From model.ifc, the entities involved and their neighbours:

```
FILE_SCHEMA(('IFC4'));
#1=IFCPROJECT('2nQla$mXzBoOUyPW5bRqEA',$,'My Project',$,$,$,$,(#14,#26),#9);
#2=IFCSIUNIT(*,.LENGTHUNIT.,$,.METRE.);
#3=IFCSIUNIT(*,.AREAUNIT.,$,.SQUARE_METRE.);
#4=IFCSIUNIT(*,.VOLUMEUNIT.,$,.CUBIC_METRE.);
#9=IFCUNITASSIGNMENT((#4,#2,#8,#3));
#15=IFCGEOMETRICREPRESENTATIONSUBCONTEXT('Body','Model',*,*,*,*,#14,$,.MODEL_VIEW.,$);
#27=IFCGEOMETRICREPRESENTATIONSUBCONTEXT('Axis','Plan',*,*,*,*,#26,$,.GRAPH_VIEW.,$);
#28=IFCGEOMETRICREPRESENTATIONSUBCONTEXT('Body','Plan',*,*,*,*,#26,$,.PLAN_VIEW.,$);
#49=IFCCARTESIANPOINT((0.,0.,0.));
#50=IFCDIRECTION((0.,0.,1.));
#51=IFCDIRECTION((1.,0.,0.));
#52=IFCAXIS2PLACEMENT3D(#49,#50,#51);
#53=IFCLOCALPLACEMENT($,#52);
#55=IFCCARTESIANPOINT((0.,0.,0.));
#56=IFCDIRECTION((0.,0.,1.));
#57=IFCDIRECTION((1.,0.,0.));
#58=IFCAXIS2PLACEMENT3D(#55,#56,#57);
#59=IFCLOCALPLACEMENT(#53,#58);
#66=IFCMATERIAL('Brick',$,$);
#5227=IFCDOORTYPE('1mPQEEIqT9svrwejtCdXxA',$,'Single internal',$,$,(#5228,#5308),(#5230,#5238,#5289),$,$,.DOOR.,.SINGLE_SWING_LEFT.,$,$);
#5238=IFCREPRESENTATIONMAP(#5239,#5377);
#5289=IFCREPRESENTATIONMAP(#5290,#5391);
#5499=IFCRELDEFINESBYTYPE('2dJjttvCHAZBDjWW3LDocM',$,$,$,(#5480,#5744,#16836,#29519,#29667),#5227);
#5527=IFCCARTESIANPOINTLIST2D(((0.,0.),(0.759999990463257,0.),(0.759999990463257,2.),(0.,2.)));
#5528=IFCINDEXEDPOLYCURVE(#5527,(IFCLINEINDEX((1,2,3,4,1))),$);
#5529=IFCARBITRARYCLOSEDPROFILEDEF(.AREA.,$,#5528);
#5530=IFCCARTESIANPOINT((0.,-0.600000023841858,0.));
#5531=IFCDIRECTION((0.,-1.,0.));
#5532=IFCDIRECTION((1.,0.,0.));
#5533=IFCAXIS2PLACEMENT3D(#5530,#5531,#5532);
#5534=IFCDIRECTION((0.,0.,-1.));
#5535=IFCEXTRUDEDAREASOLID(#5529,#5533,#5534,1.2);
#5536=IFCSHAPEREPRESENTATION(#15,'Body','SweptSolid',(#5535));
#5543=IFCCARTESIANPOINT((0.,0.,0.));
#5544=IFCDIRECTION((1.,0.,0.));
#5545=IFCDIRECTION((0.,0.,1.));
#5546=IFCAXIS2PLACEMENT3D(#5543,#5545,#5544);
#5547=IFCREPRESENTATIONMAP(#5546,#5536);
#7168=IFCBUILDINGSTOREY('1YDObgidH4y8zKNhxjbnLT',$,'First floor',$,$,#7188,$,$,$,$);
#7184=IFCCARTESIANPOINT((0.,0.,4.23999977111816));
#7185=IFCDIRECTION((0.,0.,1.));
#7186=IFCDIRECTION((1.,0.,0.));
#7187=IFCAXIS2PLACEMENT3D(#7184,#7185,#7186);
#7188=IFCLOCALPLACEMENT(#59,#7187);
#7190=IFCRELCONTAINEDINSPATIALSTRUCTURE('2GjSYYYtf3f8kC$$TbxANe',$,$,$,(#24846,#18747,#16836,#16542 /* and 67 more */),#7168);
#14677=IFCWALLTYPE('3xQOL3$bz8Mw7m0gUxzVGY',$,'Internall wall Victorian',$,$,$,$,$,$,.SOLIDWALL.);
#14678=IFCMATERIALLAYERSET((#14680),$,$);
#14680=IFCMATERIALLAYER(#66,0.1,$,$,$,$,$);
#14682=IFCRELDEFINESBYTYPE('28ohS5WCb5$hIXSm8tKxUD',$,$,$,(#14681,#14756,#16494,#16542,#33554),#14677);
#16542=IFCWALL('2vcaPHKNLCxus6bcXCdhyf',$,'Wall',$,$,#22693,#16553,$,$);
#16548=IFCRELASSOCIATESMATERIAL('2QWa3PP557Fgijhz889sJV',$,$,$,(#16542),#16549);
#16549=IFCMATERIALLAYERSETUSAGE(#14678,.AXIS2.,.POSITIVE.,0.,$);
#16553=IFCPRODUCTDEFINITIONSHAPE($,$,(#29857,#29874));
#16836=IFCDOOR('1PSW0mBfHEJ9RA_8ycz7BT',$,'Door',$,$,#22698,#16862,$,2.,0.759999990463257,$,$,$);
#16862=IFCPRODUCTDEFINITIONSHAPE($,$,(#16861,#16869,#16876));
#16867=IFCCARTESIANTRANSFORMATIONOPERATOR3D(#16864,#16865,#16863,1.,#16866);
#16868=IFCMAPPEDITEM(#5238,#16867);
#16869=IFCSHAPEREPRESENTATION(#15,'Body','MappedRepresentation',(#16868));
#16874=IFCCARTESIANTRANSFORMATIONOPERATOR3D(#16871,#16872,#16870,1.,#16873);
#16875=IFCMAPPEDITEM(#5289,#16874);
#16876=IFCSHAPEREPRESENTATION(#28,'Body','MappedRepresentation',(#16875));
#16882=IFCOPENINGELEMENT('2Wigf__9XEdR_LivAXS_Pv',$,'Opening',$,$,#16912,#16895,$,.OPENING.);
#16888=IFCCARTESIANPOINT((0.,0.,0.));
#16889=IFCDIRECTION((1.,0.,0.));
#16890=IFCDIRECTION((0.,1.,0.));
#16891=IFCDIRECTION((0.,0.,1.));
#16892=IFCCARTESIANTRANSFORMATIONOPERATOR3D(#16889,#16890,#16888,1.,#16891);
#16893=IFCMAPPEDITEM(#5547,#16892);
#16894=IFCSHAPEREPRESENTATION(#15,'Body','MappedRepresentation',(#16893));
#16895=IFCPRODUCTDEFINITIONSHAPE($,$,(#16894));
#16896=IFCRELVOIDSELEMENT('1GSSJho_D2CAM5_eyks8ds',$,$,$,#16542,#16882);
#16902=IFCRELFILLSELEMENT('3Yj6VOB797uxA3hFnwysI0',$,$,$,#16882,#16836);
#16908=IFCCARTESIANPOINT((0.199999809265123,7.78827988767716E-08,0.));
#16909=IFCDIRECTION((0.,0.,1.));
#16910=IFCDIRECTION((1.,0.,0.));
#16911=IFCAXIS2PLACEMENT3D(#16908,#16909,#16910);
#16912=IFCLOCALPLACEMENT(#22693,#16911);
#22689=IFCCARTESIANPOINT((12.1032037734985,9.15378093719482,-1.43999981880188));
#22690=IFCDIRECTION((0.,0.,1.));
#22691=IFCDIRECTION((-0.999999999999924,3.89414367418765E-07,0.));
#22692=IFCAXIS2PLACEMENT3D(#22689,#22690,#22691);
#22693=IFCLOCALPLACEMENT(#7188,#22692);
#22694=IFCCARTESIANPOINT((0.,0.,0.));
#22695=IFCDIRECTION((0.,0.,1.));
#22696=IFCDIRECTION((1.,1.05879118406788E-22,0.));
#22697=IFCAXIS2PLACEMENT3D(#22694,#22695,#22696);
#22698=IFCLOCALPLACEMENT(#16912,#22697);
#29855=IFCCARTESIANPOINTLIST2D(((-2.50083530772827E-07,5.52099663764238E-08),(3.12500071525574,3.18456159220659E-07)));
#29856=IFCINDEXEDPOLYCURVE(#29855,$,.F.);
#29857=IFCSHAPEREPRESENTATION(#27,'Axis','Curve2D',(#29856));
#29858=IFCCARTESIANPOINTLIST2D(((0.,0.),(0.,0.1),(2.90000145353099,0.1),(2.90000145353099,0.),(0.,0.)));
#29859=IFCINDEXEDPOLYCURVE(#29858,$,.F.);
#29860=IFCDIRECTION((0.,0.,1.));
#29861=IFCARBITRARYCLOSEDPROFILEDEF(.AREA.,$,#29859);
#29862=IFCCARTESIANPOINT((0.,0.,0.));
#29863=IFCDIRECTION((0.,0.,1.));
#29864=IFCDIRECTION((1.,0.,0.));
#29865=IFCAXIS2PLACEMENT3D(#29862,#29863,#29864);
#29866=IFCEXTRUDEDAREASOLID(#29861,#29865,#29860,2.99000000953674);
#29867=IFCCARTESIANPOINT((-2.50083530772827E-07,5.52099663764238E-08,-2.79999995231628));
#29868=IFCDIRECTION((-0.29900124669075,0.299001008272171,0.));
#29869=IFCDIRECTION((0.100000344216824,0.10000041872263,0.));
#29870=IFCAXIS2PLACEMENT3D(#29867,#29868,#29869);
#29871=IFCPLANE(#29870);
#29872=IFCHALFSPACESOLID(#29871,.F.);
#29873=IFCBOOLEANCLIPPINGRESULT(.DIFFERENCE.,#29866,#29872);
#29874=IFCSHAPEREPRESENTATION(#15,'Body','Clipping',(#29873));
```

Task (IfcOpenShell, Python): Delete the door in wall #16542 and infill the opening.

```python
import ifcopenshell
import ifcopenshell.api.feature
import ifcopenshell.api.root
import ifcopenshell.geom
import ifcopenshell.util.shape

model = ifcopenshell.open("model.ifc")
settings = ifcopenshell.geom.settings()


def volume(element):
    """Net volume in cubic metres, openings subtracted."""
    shape = ifcopenshell.geom.create_shape(settings, element)
    return ifcopenshell.util.shape.get_volume(shape.geometry)


door = model.by_guid("1PSW0mBfHEJ9RA_8ycz7BT")
opening = door.FillsVoids[0].RelatingOpeningElement
wall = opening.VoidsElements[0].RelatingBuildingElement
before = volume(wall)

ifcopenshell.api.root.remove_product(model, product=door)
ifcopenshell.api.feature.remove_feature(model, feature=opening)

after = volume(wall)

print(f"wall volume {before:.3f} -> {after:.3f} m3")

model.write("model_rev.ifc")
```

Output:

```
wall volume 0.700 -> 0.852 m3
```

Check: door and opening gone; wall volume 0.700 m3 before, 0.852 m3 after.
